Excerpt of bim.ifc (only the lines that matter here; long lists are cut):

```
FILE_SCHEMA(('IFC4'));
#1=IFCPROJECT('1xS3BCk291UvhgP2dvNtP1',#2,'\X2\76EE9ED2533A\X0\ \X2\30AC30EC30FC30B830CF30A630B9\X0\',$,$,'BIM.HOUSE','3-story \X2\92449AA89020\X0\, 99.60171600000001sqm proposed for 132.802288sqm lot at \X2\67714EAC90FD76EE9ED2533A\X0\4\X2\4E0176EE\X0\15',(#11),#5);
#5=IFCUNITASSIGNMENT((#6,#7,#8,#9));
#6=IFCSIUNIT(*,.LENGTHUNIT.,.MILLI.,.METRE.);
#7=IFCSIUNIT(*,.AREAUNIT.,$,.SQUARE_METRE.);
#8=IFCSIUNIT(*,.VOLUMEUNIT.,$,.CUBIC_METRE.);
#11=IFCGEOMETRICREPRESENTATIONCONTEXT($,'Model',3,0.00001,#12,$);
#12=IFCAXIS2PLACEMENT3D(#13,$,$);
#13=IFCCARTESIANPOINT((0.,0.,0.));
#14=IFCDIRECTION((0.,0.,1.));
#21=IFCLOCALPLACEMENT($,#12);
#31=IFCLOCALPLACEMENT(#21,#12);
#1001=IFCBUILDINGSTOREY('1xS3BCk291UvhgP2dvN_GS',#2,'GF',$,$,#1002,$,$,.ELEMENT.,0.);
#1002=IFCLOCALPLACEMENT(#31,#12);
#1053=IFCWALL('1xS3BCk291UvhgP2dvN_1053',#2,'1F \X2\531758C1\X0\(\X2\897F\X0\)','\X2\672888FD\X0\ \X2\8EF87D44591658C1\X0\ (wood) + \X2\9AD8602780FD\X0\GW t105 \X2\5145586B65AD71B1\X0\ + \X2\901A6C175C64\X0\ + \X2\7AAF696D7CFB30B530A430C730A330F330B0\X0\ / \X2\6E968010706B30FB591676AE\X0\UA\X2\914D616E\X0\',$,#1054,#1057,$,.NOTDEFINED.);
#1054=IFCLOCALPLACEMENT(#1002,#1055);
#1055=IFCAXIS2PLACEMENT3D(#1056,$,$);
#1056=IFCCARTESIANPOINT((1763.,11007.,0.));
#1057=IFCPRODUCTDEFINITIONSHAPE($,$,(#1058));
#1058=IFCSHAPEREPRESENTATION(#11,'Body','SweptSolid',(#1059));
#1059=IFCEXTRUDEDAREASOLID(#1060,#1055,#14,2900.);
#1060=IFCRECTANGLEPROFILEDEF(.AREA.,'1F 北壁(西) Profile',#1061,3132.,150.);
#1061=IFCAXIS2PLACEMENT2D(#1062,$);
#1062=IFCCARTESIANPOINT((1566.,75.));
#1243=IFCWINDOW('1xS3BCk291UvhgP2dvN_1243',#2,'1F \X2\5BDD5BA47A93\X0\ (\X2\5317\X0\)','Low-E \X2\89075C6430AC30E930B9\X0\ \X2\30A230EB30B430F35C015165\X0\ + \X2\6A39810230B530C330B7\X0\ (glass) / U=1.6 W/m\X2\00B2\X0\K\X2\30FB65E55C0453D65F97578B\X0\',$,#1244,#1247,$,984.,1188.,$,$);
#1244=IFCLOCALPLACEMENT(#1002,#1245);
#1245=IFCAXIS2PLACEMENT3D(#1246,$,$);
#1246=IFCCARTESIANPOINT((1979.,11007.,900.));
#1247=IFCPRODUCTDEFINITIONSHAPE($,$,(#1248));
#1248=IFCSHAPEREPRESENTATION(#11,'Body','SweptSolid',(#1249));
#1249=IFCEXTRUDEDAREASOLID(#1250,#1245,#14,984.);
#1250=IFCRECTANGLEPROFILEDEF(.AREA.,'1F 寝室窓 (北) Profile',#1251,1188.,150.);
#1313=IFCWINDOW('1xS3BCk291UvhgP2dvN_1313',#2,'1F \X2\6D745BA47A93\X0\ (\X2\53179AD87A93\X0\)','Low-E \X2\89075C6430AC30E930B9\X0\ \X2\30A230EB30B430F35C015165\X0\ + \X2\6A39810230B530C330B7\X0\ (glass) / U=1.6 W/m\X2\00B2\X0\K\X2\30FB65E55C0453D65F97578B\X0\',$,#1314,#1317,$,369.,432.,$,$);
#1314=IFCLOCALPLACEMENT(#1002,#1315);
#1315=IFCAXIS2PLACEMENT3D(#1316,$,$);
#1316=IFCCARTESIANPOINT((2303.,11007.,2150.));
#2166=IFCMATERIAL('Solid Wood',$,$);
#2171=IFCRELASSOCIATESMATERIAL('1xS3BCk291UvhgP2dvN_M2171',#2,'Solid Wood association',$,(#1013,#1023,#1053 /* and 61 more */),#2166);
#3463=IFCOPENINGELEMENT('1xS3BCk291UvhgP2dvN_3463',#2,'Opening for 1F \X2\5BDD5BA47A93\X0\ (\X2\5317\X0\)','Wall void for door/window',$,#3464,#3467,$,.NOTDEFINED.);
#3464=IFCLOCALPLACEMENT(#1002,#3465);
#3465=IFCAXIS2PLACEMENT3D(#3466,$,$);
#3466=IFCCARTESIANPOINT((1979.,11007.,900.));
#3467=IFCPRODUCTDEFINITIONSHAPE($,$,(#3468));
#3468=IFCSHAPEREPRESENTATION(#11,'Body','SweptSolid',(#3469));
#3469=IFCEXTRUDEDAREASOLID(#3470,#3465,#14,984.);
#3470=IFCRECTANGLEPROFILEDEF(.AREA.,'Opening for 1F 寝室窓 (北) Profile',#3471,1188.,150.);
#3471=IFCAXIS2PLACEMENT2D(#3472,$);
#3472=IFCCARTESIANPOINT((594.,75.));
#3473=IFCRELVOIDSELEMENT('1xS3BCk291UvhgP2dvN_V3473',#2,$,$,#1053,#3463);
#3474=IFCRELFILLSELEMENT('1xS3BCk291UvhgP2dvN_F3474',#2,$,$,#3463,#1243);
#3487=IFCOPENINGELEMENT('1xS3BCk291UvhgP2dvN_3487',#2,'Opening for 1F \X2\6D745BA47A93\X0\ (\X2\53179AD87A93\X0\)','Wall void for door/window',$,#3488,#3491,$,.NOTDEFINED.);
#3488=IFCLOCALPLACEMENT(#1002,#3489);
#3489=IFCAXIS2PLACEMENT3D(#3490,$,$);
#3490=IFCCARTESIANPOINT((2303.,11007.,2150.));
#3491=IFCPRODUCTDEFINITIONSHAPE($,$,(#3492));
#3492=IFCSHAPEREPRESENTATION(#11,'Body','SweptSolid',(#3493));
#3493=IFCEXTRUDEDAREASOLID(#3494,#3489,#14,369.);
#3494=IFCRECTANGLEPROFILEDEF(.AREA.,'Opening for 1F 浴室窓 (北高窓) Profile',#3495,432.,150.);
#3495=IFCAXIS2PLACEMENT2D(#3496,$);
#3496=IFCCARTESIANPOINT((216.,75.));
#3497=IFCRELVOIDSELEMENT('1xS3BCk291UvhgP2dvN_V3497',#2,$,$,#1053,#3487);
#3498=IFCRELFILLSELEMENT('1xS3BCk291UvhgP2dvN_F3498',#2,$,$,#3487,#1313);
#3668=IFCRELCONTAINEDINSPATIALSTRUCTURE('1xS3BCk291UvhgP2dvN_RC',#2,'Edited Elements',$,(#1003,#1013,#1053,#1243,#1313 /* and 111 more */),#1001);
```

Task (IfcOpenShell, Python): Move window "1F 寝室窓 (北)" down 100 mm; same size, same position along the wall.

```python
import numpy as np
import ifcopenshell
import ifcopenshell.api.geometry
import ifcopenshell.util.placement
import ifcopenshell.util.unit

model = ifcopenshell.open("bim.ifc")
unit_scale = ifcopenshell.util.unit.calculate_unit_scale(model)

window = model.by_guid("1xS3BCk291UvhgP2dvN_1243")
opening = window.FillsVoids[0].RelatingOpeningElement
dz = -0.1 / unit_scale

shift = np.array([0.0, 0.0, dz])
# The window is not placed relative to its opening, so move both.
for product in (opening, window):
    matrix = ifcopenshell.util.placement.get_local_placement(product.ObjectPlacement)
    matrix[:3, 3] += shift
    ifcopenshell.api.geometry.edit_object_placement(model, product=product, matrix=matrix, is_si=False)

print(f"moved by {dz * unit_scale:+.3f} m")

model.write("bim_rev.ifc")
```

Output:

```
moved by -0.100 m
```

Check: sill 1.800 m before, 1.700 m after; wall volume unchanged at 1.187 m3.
